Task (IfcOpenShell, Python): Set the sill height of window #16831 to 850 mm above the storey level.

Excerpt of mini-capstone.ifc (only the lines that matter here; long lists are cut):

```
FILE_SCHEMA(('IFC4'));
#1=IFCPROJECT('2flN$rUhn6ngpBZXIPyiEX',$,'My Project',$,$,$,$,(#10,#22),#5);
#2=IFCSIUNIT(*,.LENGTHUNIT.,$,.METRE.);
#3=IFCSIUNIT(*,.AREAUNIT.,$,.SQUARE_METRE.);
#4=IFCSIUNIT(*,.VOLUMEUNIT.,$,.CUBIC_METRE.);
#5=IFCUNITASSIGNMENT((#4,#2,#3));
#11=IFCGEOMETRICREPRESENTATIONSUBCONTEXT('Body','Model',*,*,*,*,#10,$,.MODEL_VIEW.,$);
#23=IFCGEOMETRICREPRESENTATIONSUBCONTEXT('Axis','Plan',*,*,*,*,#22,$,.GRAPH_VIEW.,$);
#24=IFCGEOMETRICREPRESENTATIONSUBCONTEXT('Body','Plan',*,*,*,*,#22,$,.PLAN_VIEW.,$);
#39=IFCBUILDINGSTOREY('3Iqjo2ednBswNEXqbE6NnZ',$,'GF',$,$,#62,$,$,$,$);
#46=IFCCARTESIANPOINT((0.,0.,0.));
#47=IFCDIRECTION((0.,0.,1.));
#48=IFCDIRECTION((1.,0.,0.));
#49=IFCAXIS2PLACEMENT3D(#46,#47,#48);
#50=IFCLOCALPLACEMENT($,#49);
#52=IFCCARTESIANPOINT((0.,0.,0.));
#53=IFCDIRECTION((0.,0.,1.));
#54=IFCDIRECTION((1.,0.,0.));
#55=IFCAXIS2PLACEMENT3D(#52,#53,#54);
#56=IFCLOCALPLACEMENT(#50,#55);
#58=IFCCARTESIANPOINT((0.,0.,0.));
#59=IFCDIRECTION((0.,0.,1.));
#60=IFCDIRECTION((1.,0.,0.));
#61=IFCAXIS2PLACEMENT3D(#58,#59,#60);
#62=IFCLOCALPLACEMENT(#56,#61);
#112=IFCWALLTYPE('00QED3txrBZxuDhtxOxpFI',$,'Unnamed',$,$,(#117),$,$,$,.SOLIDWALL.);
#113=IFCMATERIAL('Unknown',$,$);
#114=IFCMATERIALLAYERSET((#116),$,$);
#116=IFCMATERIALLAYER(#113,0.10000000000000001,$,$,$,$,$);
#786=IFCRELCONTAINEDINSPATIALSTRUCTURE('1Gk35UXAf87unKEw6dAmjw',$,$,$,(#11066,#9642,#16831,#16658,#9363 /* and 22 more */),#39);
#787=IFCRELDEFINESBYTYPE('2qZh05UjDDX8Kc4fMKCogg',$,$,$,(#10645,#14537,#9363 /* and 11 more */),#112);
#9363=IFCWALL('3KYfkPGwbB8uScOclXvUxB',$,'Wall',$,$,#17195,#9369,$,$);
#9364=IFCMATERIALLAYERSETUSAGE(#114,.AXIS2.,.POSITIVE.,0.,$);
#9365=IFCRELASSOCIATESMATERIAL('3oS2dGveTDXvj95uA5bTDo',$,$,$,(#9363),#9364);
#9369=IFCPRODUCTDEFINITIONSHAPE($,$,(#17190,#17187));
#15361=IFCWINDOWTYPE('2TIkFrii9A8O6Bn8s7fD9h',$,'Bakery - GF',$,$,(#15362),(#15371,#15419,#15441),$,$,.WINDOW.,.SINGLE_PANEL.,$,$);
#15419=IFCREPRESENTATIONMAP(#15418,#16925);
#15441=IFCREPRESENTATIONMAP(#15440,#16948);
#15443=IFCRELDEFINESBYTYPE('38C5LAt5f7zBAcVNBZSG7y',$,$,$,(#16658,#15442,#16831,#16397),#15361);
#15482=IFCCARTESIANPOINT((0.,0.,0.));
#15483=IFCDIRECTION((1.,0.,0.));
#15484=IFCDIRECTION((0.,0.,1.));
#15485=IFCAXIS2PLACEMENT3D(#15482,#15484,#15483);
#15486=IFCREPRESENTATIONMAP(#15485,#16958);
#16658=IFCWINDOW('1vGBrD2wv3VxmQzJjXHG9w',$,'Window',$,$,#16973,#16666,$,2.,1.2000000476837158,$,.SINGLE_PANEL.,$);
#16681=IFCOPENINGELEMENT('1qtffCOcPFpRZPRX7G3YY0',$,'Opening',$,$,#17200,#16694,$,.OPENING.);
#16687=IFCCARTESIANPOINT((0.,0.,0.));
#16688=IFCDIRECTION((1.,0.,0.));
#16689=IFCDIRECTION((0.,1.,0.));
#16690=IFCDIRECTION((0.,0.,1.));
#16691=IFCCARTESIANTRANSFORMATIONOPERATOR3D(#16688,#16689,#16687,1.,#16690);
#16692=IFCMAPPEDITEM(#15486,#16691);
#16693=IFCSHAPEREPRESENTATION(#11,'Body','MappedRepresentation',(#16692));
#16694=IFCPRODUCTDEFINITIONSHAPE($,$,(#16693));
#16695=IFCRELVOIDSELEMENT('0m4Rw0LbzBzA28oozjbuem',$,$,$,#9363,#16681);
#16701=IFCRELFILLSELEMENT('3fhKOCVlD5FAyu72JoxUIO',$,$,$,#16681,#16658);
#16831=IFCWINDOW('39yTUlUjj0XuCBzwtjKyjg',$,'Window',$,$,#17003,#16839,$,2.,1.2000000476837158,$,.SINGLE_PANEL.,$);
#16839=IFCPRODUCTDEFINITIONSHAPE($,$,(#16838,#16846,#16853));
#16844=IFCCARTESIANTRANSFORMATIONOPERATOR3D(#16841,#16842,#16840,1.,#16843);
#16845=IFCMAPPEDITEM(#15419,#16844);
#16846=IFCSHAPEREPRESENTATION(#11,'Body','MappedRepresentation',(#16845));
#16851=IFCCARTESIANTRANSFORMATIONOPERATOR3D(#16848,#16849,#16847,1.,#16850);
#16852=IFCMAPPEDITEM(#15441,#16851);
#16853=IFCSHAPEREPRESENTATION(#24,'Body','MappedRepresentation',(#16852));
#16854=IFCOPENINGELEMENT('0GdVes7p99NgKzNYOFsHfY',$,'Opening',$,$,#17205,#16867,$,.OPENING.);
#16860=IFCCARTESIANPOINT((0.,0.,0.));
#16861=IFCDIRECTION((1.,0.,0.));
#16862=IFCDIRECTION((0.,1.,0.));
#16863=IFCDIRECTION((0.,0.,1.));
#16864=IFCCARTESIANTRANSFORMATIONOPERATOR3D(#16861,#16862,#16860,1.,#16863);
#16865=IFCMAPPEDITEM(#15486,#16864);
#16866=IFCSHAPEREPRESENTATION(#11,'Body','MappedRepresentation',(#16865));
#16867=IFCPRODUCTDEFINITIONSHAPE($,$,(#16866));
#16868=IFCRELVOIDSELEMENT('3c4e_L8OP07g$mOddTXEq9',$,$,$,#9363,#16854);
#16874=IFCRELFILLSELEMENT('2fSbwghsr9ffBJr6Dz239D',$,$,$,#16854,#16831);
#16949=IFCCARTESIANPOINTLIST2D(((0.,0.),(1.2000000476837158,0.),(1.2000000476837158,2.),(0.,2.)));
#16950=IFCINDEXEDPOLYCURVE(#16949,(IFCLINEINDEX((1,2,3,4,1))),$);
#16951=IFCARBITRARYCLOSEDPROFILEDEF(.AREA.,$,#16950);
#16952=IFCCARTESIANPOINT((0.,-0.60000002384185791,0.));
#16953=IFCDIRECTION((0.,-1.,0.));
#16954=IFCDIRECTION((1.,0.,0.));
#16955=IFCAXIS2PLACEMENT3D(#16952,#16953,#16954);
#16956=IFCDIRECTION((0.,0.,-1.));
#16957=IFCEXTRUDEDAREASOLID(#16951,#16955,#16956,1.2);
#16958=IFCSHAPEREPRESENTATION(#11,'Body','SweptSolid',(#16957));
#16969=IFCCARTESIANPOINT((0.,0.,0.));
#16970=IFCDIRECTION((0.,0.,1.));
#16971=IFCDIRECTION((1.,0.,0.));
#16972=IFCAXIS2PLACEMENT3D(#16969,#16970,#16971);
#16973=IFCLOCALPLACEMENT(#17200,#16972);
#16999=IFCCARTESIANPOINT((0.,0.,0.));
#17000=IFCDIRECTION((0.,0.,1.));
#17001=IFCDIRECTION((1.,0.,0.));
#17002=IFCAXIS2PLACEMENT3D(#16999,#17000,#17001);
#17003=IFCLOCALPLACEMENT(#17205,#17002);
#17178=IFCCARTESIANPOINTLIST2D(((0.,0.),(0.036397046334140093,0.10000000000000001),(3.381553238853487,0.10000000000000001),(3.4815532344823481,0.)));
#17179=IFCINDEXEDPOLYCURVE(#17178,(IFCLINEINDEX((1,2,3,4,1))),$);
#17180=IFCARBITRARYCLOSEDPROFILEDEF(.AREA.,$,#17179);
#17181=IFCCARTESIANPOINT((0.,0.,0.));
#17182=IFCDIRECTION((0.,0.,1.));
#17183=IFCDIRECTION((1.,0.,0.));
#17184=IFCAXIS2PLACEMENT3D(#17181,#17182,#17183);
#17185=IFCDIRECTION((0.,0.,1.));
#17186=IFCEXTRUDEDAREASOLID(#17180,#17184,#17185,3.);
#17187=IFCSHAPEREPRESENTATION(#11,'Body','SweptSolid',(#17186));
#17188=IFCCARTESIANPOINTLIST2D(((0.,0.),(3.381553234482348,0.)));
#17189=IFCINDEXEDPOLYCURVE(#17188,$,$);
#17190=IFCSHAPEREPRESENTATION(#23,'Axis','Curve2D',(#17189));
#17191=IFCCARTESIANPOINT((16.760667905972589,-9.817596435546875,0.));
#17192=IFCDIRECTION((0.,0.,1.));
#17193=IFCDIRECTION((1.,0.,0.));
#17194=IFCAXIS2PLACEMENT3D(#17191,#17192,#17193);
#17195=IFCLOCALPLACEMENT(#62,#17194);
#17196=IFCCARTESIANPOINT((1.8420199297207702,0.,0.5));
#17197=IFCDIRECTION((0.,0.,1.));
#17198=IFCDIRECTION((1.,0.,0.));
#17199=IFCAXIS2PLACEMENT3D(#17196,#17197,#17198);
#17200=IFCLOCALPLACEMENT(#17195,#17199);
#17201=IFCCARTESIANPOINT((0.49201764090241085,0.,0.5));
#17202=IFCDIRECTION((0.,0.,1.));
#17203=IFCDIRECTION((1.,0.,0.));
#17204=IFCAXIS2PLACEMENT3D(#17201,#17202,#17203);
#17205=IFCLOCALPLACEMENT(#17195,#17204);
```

```python
import numpy as np
import ifcopenshell
import ifcopenshell.api.geometry
import ifcopenshell.geom
import ifcopenshell.util.element
import ifcopenshell.util.placement
import ifcopenshell.util.shape
import ifcopenshell.util.unit

model = ifcopenshell.open("mini-capstone.ifc")
unit_scale = ifcopenshell.util.unit.calculate_unit_scale(model)

window = model.by_guid("39yTUlUjj0XuCBzwtjKyjg")
opening = window.FillsVoids[0].RelatingOpeningElement
storey = ifcopenshell.util.element.get_container(window, ifc_class="IfcBuildingStorey")
level = ifcopenshell.util.placement.get_local_placement(storey.ObjectPlacement)[2, 3]

# The opening's origin need not be at the sill, so measure its lowest point.
shape = ifcopenshell.geom.create_shape(ifcopenshell.geom.settings(), opening)
bottom = ifcopenshell.util.shape.get_shape_bottom_elevation(shape, shape.geometry) / unit_scale
dz = level + 0.85 / unit_scale - bottom

shift = np.array([0.0, 0.0, dz])
# The window is placed relative to its opening, so it follows when the opening moves.
matrix = ifcopenshell.util.placement.get_local_placement(opening.ObjectPlacement)
matrix[:3, 3] += shift
ifcopenshell.api.geometry.edit_object_placement(
    model, product=opening, matrix=matrix, is_si=False, should_transform_children=True
)

print(f"moved by {dz * unit_scale:+.3f} m")

model.write("mini-capstone_v2.ifc")
```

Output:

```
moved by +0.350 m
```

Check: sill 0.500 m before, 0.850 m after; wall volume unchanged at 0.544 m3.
